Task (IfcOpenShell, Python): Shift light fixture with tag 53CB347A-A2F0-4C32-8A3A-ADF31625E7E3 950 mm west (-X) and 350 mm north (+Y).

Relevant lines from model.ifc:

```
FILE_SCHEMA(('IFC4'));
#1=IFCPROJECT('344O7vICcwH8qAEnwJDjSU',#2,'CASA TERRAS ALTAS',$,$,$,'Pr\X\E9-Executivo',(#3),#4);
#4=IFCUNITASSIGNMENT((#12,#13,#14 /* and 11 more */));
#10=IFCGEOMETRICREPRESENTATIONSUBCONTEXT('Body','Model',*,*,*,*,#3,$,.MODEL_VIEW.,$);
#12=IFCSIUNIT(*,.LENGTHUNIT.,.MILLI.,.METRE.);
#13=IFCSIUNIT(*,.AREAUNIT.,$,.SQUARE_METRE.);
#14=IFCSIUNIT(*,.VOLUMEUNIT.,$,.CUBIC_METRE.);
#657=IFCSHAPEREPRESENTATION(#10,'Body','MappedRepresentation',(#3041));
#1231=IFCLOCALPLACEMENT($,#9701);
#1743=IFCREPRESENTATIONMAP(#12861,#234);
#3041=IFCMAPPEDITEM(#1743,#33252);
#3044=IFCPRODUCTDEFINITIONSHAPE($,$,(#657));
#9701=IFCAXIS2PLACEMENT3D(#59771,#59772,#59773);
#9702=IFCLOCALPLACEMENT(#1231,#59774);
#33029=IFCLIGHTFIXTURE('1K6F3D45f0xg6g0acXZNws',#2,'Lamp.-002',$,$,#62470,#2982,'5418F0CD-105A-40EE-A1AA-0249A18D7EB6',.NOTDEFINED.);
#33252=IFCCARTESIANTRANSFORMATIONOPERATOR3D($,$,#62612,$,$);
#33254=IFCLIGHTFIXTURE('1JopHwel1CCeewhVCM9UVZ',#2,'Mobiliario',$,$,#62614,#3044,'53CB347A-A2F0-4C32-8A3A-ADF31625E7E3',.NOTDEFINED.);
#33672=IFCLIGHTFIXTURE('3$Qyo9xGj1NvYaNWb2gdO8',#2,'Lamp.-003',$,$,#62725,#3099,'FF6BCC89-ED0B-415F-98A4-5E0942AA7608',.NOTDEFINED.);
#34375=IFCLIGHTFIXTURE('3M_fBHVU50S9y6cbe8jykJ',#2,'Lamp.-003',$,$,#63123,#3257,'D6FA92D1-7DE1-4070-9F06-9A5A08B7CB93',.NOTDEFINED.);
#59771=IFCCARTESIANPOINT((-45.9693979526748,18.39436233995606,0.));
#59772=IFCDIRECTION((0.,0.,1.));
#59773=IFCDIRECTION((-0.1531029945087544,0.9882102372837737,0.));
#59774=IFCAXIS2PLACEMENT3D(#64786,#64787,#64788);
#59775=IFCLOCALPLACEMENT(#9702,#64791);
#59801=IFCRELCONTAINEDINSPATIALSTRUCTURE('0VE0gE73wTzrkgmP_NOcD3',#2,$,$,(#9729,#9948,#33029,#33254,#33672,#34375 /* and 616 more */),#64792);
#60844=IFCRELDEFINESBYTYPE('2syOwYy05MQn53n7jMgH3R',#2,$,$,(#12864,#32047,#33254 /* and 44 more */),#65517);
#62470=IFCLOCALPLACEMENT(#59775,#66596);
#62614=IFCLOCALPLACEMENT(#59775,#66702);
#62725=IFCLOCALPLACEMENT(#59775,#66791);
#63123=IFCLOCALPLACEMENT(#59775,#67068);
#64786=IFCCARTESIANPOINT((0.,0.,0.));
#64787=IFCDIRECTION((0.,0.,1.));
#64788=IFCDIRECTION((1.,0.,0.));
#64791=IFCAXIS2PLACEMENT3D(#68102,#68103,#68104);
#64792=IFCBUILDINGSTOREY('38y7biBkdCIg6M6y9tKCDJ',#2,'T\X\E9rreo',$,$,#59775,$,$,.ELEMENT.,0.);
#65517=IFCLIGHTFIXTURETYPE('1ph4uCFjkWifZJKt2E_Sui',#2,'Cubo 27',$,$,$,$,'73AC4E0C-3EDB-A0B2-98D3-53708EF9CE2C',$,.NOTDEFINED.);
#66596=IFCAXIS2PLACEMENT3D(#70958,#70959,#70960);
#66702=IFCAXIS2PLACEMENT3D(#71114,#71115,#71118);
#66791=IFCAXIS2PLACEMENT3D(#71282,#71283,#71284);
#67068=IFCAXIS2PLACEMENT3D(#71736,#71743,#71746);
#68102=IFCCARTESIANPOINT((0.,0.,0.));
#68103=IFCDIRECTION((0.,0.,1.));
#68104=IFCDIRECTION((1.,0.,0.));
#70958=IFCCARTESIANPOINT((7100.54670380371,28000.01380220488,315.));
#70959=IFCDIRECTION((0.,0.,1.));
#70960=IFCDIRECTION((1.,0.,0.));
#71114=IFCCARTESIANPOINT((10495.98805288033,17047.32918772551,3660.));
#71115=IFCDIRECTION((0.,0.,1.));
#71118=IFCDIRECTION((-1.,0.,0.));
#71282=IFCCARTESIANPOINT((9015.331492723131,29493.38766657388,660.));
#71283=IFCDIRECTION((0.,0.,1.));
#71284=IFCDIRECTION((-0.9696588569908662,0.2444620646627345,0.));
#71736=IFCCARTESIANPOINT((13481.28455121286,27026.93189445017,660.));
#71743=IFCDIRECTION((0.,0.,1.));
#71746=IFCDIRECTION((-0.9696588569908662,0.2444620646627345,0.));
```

```python
import ifcopenshell
import ifcopenshell.api.geometry
import ifcopenshell.util.placement
import ifcopenshell.util.unit

model = ifcopenshell.open("model.ifc")
unit_scale = ifcopenshell.util.unit.calculate_unit_scale(model)

item = model.by_id(33254)
matrix = ifcopenshell.util.placement.get_local_placement(item.ObjectPlacement)
matrix[0, 3] -= 0.95 / unit_scale
matrix[1, 3] += 0.35 / unit_scale
ifcopenshell.api.geometry.edit_object_placement(model, product=item, matrix=matrix, is_si=False)

print(ifcopenshell.util.placement.get_local_placement(item.ObjectPlacement).round(3) + 0.0)

model.write("model_rev.ifc")
```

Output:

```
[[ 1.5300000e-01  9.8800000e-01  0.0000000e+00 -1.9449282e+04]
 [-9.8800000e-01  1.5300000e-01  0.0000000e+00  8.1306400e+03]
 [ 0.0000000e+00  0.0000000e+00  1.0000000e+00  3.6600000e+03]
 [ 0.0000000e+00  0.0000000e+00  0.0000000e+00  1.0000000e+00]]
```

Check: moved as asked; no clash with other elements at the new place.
